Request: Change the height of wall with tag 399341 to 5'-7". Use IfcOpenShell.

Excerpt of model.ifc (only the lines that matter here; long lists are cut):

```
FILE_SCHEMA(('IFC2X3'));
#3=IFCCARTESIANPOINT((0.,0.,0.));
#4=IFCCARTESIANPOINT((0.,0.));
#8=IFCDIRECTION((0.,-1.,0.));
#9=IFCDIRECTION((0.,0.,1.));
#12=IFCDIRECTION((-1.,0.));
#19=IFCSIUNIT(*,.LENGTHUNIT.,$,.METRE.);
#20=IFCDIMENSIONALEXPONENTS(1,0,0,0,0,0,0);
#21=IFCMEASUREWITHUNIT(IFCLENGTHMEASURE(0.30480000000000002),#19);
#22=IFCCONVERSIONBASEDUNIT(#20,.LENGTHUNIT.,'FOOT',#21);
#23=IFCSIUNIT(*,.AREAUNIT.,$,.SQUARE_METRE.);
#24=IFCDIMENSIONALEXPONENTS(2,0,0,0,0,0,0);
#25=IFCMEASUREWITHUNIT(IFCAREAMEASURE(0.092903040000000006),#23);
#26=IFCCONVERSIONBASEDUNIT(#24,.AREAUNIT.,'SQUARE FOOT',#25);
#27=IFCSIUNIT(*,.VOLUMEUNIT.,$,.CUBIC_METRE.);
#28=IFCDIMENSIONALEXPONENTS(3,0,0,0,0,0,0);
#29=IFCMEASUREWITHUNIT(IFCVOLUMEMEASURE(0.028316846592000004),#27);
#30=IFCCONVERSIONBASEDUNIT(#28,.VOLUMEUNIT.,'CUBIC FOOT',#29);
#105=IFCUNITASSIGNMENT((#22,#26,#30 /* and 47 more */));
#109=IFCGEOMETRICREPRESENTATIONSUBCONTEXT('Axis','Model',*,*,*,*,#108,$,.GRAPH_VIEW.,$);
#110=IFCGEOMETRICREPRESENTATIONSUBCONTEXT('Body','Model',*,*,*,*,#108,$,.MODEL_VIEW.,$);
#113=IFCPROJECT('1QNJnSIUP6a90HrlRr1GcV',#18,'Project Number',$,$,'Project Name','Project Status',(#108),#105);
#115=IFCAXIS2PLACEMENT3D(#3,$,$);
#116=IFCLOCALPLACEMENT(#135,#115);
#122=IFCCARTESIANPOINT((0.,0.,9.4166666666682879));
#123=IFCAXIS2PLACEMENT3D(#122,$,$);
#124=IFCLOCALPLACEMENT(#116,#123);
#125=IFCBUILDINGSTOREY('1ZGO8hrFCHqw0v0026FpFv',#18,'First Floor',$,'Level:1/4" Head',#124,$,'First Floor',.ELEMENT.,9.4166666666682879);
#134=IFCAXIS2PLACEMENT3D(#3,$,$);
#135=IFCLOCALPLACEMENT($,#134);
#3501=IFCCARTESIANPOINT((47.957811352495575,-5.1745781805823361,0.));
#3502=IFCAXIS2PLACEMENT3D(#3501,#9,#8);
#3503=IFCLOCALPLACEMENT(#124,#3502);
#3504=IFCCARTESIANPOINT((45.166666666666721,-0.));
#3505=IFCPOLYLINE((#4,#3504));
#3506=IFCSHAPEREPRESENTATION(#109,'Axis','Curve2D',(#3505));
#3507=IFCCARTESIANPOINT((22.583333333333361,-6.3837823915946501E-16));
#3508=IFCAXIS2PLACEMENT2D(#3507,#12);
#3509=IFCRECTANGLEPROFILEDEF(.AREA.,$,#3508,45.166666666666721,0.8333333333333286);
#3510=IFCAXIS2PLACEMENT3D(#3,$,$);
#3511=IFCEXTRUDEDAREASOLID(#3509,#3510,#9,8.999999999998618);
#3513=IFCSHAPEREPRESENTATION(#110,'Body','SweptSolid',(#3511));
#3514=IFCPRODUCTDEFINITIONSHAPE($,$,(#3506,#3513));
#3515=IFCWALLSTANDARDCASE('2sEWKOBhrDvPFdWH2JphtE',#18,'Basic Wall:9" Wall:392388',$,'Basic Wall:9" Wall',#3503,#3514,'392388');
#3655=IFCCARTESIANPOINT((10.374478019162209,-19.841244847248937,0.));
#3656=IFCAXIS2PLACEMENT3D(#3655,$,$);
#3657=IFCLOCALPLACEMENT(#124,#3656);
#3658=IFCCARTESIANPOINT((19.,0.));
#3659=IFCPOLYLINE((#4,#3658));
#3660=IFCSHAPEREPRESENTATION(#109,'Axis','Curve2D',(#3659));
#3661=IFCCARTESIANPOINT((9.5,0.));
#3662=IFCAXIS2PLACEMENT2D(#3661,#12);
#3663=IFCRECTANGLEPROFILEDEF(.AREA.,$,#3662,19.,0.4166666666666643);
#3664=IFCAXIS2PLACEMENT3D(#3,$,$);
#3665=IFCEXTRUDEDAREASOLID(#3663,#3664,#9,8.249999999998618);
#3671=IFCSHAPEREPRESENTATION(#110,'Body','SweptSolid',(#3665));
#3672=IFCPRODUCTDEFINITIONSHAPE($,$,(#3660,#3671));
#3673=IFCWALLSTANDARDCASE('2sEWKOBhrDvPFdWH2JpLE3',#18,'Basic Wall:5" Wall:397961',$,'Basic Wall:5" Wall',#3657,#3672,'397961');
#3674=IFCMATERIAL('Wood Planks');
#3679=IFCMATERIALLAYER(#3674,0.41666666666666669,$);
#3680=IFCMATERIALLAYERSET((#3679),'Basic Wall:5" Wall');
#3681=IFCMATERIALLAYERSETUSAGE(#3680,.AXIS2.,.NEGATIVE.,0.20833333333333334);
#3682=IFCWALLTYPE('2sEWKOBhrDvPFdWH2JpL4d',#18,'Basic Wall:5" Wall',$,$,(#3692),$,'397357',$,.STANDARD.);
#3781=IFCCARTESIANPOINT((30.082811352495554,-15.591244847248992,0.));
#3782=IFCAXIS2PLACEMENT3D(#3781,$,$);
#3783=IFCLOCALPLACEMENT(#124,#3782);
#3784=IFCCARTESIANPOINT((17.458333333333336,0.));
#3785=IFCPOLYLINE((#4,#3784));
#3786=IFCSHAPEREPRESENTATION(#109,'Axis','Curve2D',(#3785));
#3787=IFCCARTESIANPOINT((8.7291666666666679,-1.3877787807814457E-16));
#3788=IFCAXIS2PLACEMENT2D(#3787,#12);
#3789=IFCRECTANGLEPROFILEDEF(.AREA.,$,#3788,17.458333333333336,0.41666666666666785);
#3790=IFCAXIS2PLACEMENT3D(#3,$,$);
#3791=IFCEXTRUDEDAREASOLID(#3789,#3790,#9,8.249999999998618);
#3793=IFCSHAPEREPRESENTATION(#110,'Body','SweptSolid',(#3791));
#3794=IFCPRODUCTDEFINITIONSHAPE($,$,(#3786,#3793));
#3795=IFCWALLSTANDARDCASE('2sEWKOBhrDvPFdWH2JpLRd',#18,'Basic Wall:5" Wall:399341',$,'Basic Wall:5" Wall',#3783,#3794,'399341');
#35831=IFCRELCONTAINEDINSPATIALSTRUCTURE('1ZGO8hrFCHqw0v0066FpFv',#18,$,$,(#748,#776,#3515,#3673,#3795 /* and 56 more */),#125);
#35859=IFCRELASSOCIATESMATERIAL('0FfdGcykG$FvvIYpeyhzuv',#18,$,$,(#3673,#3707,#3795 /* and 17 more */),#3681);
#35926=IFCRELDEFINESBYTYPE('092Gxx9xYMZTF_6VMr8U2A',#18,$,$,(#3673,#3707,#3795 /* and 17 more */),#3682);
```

```python
import ifcopenshell
import ifcopenshell.geom
import ifcopenshell.util.representation
import ifcopenshell.util.shape
import ifcopenshell.util.unit

model = ifcopenshell.open("model.ifc")
unit_scale = ifcopenshell.util.unit.calculate_unit_scale(model)
settings = ifcopenshell.geom.settings()


def volume(element):
    """Net volume in cubic metres, openings subtracted."""
    shape = ifcopenshell.geom.create_shape(settings, element)
    return ifcopenshell.util.shape.get_volume(shape.geometry)


wall = model.by_guid("2sEWKOBhrDvPFdWH2JpLRd")
before = volume(wall)

body = ifcopenshell.util.representation.get_representation(wall, "Model", "Body")
solid = body.Items[0]
old_height = solid.Depth
solid.Depth = 67 * 0.0254 / unit_scale
after = volume(wall)

print(f"height {old_height:g} -> {solid.Depth:g}, volume {before:.3f} -> {after:.3f} m3")

model.write("model_updated.ifc")
```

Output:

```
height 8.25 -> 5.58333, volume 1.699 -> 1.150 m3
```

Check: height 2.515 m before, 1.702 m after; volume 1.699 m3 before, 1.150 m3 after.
